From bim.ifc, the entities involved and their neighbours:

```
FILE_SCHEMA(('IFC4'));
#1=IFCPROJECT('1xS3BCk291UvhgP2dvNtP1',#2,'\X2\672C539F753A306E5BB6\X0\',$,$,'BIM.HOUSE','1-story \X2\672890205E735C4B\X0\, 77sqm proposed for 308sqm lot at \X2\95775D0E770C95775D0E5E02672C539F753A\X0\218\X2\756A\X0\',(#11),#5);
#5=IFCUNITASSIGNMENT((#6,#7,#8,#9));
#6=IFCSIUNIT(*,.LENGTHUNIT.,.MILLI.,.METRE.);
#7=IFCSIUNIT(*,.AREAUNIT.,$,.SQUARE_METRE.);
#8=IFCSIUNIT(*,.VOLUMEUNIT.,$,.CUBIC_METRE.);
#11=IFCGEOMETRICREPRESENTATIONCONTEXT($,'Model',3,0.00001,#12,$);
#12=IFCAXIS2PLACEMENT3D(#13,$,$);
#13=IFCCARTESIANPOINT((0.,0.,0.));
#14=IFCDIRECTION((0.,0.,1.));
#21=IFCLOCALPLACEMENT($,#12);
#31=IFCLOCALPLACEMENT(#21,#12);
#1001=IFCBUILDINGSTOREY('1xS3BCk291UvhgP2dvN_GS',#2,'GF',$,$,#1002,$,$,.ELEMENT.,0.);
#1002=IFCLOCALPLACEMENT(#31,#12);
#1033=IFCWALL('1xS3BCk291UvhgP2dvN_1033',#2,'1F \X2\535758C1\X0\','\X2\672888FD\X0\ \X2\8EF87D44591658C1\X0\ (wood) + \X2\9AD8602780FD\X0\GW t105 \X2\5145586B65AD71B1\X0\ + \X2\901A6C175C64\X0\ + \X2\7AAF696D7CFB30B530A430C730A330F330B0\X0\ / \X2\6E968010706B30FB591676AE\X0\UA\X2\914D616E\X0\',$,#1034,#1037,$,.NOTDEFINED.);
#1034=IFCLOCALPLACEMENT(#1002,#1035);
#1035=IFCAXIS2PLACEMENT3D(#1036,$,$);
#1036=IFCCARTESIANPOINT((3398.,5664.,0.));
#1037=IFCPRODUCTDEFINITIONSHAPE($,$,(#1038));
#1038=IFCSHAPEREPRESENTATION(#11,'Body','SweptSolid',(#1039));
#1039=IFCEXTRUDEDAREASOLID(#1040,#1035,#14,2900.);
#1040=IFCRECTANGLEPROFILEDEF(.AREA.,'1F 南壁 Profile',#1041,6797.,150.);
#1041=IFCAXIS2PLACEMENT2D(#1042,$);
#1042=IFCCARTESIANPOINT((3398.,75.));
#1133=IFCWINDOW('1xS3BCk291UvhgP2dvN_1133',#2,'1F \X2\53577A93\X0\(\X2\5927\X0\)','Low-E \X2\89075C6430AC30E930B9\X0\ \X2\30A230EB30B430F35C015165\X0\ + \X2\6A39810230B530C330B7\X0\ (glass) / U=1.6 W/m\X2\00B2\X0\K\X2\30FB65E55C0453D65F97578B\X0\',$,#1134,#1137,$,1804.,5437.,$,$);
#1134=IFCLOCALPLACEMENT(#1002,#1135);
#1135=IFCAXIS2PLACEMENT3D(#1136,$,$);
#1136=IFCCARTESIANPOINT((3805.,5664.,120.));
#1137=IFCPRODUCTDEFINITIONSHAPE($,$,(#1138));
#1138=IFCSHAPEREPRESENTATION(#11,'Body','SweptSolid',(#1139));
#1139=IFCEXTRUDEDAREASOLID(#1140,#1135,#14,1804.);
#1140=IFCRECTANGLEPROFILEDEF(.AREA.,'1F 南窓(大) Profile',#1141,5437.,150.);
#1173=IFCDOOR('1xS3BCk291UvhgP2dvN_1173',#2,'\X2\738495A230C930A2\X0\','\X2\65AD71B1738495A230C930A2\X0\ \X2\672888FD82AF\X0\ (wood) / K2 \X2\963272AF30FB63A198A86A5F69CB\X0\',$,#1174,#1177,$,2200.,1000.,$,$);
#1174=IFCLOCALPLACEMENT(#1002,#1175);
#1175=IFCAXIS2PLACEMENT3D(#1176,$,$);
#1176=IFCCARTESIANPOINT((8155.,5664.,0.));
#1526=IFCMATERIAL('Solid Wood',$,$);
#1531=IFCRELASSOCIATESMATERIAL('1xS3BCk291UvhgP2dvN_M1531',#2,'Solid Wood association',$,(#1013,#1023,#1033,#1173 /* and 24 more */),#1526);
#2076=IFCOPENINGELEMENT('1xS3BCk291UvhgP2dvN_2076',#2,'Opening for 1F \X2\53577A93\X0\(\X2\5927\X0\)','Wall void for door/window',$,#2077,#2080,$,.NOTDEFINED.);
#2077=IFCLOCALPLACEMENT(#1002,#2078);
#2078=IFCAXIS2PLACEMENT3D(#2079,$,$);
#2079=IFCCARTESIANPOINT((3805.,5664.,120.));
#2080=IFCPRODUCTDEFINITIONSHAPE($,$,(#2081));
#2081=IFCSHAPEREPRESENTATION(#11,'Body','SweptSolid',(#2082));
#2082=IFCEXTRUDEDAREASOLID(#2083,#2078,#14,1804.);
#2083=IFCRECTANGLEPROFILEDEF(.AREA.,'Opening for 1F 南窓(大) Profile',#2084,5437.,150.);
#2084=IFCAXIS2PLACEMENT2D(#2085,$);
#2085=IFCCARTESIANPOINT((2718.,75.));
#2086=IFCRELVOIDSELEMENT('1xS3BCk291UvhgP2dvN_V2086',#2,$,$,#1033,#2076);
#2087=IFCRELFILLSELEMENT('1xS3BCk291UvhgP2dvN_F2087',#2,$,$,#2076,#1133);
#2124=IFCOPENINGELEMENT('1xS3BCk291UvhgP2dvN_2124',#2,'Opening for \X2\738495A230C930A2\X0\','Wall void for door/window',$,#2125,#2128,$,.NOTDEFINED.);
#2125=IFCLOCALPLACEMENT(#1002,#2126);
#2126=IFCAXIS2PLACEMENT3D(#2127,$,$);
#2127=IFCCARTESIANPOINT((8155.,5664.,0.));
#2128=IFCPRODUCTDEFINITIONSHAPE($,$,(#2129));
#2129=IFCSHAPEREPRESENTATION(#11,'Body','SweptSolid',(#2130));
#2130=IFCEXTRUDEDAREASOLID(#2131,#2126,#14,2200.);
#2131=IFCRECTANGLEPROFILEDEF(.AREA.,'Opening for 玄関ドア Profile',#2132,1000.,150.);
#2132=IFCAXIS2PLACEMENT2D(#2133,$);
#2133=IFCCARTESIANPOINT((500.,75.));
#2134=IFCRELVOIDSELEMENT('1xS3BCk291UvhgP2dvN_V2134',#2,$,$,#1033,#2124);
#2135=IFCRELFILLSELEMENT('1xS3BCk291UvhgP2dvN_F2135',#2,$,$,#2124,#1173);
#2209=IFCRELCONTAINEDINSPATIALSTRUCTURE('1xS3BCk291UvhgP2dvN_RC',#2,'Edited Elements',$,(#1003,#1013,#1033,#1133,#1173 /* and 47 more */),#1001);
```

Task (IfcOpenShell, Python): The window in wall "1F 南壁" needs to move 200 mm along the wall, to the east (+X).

```python
import ifcopenshell
import ifcopenshell.api.geometry
import ifcopenshell.util.placement

model = ifcopenshell.open("bim.ifc")

window = model.by_id(1133)
opening = window.FillsVoids[0].RelatingOpeningElement
wall = opening.VoidsElements[0].RelatingBuildingElement

wall_matrix = ifcopenshell.util.placement.get_local_placement(wall.ObjectPlacement)
shift = wall_matrix[:3, 0] * 200.0
before = ifcopenshell.util.placement.get_local_placement(window.ObjectPlacement)[:3, 3].copy()

# The window is not placed relative to its opening, so move both.
for product in (opening, window):
    matrix = ifcopenshell.util.placement.get_local_placement(product.ObjectPlacement)
    matrix[:3, 3] += shift
    ifcopenshell.api.geometry.edit_object_placement(model, product=product, matrix=matrix, is_si=False)

after = ifcopenshell.util.placement.get_local_placement(window.ObjectPlacement)[:3, 3]
print("window moved by", (after - before).round(3) + 0.0)

model.write("bim_updated.ifc")
```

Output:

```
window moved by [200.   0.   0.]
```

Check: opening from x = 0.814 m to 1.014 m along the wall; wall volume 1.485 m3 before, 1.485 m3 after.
